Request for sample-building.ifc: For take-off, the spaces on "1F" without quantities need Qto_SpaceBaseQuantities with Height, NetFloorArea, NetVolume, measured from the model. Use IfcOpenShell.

First a look at what the model holds.

```python
import ifcopenshell
import ifcopenshell.util.element
import ifcopenshell.util.unit

model = ifcopenshell.open("sample-building.ifc")
print(model.schema)
for unit_type in ("LENGTHUNIT", "AREAUNIT", "VOLUMEUNIT"):
    print(unit_type, ifcopenshell.util.unit.calculate_unit_scale(model, unit_type))
storey = next(s for s in model.by_type("IfcBuildingStorey") if s.Name == "1F")
spaces = [e for e in ifcopenshell.util.element.get_decomposition(storey) if e.is_a("IfcSpace")]
for e in sorted(spaces, key=lambda e: e.id()):
    print(e.id(), e.is_a(), e.Name, list(ifcopenshell.util.element.get_psets(e, qtos_only=True)), sep=" | ")
```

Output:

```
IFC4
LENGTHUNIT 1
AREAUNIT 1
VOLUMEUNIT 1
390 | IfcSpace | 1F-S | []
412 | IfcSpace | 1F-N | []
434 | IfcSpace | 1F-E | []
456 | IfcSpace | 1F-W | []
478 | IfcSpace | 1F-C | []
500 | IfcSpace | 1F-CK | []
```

```python
import ifcopenshell
import ifcopenshell.api.pset
import ifcopenshell.geom
import ifcopenshell.util.element
import ifcopenshell.util.shape
import ifcopenshell.util.unit

model = ifcopenshell.open("sample-building.ifc")
unit_scale = ifcopenshell.util.unit.calculate_unit_scale(model)
area_scale = ifcopenshell.util.unit.calculate_unit_scale(model, "AREAUNIT")
volume_scale = ifcopenshell.util.unit.calculate_unit_scale(model, "VOLUMEUNIT")
settings = ifcopenshell.geom.settings()

storey = next(s for s in model.by_type("IfcBuildingStorey") if s.Name == "1F")
spaces = [e for e in ifcopenshell.util.element.get_decomposition(storey) if e.is_a("IfcSpace")]

for e in sorted(spaces, key=lambda e: e.id()):
    if ifcopenshell.util.element.get_psets(e, qtos_only=True, should_inherit=False):
        continue
    # Geometry comes back in metres, in the element's own axes.
    shape = ifcopenshell.geom.create_shape(settings, e)
    values = {
        "Height": ifcopenshell.util.shape.get_z(shape.geometry) / unit_scale,
        "NetFloorArea": ifcopenshell.util.shape.get_footprint_area(shape.geometry) / area_scale,
        "NetVolume": ifcopenshell.util.shape.get_volume(shape.geometry) / volume_scale,
    }
    qto = ifcopenshell.api.pset.add_qto(model, product=e, name="Qto_SpaceBaseQuantities")
    ifcopenshell.api.pset.edit_qto(model, qto=qto, properties=values)
    print(e.id(), {k: round(v, 3) for k, v in values.items()})

model.write("sample-building_edited.ifc")
```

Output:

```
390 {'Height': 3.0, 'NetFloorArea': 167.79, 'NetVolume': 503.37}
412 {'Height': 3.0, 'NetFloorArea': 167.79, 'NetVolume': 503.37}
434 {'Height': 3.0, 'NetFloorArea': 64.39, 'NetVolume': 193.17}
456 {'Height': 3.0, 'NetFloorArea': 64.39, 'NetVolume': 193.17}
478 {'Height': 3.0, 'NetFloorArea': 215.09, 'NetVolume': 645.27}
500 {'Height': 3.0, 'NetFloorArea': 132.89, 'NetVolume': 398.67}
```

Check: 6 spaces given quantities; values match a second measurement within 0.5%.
